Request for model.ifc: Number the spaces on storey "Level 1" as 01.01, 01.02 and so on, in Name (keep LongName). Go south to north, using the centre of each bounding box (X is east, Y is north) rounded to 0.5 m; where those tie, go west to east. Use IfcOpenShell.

First a look at what the model holds.

```python
import ifcopenshell
import ifcopenshell.util.element
import ifcopenshell.util.placement

model = ifcopenshell.open("model.ifc")
print(model.schema)
storey = next(s for s in model.by_type("IfcBuildingStorey") if s.Name == "Level 1")
spaces = [e for e in ifcopenshell.util.element.get_decomposition(storey) if e.is_a("IfcSpace")]
for e in sorted(spaces, key=lambda e: e.id()):
    origin = ifcopenshell.util.placement.get_local_placement(e.ObjectPlacement)[:3, 3]
    print(e.id(), e.Name, e.LongName, origin.round(2) + 0.0, sep=" | ")
```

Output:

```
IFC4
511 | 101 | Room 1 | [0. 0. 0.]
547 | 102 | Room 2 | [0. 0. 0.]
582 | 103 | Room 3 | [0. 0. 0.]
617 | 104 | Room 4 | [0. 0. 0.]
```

```python
import ifcopenshell
import ifcopenshell.geom
import ifcopenshell.util.element
import ifcopenshell.util.shape

model = ifcopenshell.open("model.ifc")
settings = ifcopenshell.geom.settings()
settings.set("use-world-coords", True)


def centre(element):
    shape = ifcopenshell.geom.create_shape(settings, element)
    return ifcopenshell.util.shape.get_bbox_centroid(shape.geometry)


storey = next(s for s in model.by_type("IfcBuildingStorey") if s.Name == "Level 1")
spaces = [e for e in ifcopenshell.util.element.get_decomposition(storey) if e.is_a("IfcSpace")]

# Insertion points can sit at a corner or the storey origin, so sort by the geometry (in metres).
centres = {e: centre(e) for e in spaces}
spaces.sort(key=lambda e: (round(centres[e][1] / 0.5), centres[e][0]))

for i, e in enumerate(spaces, start=1):
    number = f"01.{i:02d}"
    e.Name = number
    print(e.id(), number)

model.write("model_v2.ifc")
```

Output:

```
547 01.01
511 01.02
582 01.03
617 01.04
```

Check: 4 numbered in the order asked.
